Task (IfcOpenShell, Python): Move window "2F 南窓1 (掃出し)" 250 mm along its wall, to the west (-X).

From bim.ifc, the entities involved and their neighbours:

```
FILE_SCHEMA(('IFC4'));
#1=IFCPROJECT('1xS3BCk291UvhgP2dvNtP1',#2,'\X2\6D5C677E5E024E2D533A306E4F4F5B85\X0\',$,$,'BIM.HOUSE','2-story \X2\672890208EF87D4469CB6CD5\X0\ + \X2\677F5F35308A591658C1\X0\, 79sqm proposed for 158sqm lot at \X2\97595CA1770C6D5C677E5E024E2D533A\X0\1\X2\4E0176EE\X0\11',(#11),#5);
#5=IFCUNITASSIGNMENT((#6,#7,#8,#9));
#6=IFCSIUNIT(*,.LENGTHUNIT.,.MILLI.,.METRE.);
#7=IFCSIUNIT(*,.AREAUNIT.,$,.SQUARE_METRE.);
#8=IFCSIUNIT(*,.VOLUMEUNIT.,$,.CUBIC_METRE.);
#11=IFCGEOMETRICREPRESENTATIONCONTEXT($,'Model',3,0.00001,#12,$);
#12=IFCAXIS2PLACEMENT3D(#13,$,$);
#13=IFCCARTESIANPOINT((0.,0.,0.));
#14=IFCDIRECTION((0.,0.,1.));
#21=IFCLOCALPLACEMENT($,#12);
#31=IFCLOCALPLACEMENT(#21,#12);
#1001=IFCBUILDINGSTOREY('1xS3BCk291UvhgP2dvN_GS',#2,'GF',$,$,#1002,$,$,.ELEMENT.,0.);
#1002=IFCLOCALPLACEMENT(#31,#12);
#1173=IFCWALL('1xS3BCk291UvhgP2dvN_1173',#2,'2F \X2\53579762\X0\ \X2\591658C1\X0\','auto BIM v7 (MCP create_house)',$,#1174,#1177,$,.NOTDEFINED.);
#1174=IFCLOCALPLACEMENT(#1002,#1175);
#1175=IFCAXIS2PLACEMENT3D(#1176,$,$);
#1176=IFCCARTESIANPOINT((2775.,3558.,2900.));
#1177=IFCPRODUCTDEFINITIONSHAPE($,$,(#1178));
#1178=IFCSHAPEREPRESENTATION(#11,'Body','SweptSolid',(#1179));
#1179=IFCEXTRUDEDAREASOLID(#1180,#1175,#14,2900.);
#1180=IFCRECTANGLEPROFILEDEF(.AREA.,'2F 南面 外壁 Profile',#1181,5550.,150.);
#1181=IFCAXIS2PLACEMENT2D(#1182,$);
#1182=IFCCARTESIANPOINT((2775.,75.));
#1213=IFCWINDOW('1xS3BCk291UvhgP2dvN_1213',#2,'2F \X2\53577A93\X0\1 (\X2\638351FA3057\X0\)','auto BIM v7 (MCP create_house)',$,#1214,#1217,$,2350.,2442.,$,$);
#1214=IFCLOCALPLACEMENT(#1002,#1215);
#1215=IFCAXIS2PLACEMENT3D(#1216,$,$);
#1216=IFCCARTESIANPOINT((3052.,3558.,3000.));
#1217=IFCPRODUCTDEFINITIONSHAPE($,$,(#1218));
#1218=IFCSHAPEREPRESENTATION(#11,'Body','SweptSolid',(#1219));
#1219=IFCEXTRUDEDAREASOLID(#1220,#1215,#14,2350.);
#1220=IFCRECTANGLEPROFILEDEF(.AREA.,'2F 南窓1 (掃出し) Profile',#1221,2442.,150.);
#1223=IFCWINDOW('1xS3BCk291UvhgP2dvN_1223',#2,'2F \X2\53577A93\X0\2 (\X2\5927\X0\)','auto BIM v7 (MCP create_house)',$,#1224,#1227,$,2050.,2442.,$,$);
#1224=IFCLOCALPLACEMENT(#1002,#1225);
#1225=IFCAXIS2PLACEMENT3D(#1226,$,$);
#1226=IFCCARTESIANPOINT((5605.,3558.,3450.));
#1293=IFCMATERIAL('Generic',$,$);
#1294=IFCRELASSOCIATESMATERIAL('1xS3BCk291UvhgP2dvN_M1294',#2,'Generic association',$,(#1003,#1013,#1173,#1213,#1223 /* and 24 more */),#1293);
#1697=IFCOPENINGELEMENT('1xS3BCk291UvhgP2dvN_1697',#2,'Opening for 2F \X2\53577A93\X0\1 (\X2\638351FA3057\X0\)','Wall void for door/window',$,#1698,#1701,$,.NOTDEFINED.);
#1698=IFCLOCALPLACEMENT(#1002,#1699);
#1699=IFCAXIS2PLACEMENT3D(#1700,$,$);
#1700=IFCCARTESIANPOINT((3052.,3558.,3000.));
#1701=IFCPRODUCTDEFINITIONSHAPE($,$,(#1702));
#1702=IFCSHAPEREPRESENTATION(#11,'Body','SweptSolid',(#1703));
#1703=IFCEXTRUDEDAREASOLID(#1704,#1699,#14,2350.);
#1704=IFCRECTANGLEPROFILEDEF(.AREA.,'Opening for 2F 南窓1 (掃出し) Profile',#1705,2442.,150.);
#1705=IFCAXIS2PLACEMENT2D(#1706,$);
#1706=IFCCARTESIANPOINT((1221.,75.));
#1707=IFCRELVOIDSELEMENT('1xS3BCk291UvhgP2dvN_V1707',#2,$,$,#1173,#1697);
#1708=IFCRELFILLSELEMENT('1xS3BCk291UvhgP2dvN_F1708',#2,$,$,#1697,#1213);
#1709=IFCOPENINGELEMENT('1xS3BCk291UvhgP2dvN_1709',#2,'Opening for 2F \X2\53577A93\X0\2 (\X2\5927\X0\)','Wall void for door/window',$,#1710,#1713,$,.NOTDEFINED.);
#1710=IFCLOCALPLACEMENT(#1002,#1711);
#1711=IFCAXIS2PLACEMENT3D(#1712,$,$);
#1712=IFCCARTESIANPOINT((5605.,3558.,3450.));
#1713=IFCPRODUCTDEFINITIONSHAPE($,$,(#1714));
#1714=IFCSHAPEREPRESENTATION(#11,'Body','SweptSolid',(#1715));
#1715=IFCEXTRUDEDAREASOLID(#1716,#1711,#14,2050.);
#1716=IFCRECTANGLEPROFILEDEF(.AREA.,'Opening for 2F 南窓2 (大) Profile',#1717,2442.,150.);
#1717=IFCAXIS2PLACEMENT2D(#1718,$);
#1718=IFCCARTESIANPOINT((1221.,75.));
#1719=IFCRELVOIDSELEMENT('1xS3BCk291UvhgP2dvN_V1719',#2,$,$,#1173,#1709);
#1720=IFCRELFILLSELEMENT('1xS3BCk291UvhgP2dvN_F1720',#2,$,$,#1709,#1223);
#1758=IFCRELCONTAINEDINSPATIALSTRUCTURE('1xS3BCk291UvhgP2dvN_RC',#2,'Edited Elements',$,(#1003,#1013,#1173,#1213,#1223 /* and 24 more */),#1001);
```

```python
import ifcopenshell
import ifcopenshell.api.geometry
import ifcopenshell.util.placement
import ifcopenshell.util.unit

model = ifcopenshell.open("bim.ifc")
unit_scale = ifcopenshell.util.unit.calculate_unit_scale(model)

window = model.by_id(1213)
opening = window.FillsVoids[0].RelatingOpeningElement
wall = opening.VoidsElements[0].RelatingBuildingElement

wall_matrix = ifcopenshell.util.placement.get_local_placement(wall.ObjectPlacement)
shift = wall_matrix[:3, 0] * -0.25 / unit_scale
before = ifcopenshell.util.placement.get_local_placement(window.ObjectPlacement)[:3, 3].copy()

# The window is not placed relative to its opening, so move both.
for product in (opening, window):
    matrix = ifcopenshell.util.placement.get_local_placement(product.ObjectPlacement)
    matrix[:3, 3] += shift
    ifcopenshell.api.geometry.edit_object_placement(model, product=product, matrix=matrix, is_si=False)

after = ifcopenshell.util.placement.get_local_placement(window.ObjectPlacement)[:3, 3]
print("window moved by", (after - before).round(3) + 0.0)

model.write("bim_v2.ifc")
```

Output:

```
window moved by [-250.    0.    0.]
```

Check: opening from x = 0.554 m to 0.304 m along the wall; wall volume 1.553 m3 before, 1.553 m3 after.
